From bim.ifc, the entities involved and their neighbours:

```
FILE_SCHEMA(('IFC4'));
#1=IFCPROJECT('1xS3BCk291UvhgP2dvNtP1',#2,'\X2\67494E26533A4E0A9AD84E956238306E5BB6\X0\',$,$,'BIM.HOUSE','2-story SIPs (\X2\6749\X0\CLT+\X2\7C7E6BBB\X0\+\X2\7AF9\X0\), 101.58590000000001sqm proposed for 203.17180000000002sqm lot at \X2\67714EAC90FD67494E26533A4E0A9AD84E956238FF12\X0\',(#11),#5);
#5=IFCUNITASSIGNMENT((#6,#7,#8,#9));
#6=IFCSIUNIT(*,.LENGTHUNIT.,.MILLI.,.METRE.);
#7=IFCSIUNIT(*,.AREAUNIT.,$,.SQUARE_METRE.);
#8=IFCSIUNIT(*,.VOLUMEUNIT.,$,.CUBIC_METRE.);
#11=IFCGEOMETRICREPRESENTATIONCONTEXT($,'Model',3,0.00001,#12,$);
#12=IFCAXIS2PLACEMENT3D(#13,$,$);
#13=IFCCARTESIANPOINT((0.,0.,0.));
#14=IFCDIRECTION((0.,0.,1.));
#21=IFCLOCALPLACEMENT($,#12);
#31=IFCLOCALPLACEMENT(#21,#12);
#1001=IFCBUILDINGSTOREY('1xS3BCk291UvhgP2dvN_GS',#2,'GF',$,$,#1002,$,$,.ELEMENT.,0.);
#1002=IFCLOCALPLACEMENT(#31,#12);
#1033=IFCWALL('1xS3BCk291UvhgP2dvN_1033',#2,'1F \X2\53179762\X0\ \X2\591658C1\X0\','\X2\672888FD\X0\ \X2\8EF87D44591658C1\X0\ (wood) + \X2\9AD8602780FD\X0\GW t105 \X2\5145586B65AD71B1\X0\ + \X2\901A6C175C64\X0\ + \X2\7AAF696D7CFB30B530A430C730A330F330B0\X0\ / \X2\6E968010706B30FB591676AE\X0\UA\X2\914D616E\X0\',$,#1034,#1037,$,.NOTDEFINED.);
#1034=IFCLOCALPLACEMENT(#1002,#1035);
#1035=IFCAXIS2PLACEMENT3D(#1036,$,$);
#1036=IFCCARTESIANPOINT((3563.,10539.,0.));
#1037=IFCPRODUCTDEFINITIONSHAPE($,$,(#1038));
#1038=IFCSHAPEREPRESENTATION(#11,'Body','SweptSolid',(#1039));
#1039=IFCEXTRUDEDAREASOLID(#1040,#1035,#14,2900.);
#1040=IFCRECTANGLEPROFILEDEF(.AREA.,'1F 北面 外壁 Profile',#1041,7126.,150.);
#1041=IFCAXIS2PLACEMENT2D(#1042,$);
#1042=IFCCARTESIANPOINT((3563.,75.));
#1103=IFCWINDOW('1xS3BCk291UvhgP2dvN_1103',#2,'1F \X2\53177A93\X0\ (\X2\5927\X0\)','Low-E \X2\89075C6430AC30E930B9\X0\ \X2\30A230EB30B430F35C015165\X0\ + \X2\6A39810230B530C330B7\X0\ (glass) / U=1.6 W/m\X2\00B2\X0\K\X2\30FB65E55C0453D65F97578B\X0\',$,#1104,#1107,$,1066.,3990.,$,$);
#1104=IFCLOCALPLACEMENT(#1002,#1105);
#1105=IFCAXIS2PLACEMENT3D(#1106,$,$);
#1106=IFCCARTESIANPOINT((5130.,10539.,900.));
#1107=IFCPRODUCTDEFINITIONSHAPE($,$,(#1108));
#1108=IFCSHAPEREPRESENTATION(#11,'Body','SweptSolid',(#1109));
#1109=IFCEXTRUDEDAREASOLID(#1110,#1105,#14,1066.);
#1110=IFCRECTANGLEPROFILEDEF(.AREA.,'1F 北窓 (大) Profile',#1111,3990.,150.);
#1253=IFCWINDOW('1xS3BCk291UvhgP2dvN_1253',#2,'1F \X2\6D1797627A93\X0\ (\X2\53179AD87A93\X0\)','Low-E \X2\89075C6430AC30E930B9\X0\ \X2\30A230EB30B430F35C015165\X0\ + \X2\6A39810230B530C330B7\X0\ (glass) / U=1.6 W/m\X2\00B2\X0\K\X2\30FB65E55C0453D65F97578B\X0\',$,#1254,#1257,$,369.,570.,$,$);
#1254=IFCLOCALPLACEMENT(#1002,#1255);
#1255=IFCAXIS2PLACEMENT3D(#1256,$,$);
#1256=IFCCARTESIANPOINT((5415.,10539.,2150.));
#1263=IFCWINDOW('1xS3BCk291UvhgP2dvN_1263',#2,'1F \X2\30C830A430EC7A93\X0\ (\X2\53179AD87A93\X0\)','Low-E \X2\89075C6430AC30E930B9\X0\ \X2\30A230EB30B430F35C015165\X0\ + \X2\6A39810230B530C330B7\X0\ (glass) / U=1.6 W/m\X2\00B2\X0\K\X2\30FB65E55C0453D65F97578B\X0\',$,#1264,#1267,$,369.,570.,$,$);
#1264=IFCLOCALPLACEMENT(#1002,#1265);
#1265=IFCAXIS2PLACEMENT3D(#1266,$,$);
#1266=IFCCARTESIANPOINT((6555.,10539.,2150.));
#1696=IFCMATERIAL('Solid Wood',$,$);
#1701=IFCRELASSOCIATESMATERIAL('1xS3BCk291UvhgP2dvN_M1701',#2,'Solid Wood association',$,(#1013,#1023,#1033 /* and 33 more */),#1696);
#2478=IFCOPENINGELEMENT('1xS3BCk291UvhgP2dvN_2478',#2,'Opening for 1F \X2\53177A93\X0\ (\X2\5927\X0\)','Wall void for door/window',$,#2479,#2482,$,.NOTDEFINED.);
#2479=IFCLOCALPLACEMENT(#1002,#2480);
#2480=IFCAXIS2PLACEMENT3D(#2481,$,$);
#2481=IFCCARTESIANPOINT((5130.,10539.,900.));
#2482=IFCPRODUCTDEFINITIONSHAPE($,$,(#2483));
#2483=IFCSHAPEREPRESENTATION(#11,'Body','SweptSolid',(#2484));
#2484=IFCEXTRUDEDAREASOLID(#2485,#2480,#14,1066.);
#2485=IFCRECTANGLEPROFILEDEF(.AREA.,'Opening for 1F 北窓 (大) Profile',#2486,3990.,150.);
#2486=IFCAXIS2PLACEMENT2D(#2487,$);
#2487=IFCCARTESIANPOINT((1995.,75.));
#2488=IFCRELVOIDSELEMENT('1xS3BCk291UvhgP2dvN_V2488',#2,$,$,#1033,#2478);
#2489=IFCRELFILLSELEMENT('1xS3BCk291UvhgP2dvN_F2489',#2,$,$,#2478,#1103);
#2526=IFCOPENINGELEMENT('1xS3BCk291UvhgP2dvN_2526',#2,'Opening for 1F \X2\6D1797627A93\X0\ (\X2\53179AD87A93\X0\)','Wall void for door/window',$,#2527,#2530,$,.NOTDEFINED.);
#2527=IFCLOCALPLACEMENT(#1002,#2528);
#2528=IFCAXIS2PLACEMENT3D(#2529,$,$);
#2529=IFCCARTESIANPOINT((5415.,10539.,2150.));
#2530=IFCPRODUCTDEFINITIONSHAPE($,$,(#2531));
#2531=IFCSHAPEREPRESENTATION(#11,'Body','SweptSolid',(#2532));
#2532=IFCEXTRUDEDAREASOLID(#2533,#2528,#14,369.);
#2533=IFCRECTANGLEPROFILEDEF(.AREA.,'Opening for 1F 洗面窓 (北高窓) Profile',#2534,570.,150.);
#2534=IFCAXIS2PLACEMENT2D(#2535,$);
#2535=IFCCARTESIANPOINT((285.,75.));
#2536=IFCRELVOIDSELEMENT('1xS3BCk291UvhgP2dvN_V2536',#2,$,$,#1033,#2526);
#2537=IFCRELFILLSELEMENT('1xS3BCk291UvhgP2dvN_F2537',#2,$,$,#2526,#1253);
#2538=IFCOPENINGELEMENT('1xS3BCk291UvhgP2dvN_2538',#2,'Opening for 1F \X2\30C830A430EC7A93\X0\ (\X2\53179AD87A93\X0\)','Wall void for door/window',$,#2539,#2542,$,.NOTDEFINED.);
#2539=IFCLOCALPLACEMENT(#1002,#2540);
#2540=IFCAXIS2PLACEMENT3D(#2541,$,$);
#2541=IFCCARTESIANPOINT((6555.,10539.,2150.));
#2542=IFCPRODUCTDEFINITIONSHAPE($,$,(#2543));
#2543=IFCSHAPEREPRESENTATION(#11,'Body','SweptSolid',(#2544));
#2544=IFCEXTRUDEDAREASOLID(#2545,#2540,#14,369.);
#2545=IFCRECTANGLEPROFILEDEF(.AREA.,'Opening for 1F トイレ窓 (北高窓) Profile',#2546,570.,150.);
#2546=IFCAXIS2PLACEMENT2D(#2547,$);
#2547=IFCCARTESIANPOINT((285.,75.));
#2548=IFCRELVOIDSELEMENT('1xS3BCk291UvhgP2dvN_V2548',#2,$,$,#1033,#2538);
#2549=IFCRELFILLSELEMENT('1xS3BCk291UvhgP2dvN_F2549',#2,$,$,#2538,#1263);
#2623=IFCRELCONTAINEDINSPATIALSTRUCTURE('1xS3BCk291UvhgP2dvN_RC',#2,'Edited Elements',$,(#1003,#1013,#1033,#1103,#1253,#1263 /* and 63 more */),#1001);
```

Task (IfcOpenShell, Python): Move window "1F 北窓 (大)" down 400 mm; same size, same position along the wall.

```python
import numpy as np
import ifcopenshell
import ifcopenshell.api.geometry
import ifcopenshell.util.placement
import ifcopenshell.util.unit

model = ifcopenshell.open("bim.ifc")
unit_scale = ifcopenshell.util.unit.calculate_unit_scale(model)

window = model.by_guid("1xS3BCk291UvhgP2dvN_1103")
opening = window.FillsVoids[0].RelatingOpeningElement
dz = -0.4 / unit_scale

shift = np.array([0.0, 0.0, dz])
# The window is not placed relative to its opening, so move both.
for product in (opening, window):
    matrix = ifcopenshell.util.placement.get_local_placement(product.ObjectPlacement)
    matrix[:3, 3] += shift
    ifcopenshell.api.geometry.edit_object_placement(model, product=product, matrix=matrix, is_si=False)

print(f"moved by {dz * unit_scale:+.3f} m")

model.write("bim-out.ifc")
```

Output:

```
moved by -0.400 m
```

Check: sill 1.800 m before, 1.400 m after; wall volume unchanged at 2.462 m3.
